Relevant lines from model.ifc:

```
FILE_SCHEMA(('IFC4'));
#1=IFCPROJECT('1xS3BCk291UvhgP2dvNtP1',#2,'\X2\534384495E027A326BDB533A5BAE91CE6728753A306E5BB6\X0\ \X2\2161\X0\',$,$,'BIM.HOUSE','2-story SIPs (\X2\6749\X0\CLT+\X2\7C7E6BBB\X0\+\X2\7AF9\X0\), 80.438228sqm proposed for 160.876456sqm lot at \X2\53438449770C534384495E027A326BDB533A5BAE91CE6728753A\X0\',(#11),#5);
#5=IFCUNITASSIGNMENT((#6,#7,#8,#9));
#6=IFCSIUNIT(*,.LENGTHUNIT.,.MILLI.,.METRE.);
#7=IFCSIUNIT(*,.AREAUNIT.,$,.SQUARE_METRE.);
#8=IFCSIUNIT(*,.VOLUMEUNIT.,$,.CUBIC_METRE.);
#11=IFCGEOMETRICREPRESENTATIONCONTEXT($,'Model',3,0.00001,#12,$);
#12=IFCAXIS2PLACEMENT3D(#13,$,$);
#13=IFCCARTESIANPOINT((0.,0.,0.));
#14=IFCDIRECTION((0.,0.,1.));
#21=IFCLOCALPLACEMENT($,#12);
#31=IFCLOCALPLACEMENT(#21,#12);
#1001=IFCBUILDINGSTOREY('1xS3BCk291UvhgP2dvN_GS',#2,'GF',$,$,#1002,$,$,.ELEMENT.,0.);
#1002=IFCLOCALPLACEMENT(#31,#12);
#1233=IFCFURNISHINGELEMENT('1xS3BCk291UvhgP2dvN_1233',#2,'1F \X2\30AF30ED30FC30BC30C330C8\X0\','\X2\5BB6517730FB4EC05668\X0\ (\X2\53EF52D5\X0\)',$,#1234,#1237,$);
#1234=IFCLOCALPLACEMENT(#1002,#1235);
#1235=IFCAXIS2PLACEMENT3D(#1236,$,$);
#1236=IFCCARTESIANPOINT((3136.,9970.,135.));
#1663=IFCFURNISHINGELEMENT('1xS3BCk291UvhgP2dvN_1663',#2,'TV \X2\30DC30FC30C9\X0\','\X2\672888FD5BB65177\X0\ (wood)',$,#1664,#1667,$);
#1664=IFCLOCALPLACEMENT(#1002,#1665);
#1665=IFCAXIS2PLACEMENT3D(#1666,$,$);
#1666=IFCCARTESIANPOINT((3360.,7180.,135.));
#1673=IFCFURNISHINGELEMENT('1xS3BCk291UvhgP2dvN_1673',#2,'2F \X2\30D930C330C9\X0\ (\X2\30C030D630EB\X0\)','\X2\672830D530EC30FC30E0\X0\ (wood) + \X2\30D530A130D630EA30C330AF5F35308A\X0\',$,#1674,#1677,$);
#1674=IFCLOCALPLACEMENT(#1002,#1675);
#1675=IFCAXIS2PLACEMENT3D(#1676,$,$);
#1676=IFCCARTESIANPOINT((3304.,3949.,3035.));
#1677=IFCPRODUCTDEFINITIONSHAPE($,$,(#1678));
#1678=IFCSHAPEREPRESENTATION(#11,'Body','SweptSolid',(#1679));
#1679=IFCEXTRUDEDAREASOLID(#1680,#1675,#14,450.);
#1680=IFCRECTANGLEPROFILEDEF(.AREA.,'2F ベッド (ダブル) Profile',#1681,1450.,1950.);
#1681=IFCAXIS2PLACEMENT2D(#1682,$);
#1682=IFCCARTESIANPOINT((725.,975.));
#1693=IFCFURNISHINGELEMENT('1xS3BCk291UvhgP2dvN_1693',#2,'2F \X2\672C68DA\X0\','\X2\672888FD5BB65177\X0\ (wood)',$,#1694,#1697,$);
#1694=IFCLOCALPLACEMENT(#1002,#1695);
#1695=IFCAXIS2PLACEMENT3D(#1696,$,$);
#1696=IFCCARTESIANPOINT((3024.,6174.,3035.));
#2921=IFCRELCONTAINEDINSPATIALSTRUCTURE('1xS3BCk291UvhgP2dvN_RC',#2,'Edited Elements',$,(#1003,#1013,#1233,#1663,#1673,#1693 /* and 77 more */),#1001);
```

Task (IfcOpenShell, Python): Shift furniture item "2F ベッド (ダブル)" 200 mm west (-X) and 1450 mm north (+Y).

```python
import ifcopenshell
import ifcopenshell.api.geometry
import ifcopenshell.util.placement
import ifcopenshell.util.unit

model = ifcopenshell.open("model.ifc")
unit_scale = ifcopenshell.util.unit.calculate_unit_scale(model)

item = model.by_guid("1xS3BCk291UvhgP2dvN_1673")
matrix = ifcopenshell.util.placement.get_local_placement(item.ObjectPlacement)
matrix[0, 3] -= 0.2 / unit_scale
matrix[1, 3] += 1.45 / unit_scale
ifcopenshell.api.geometry.edit_object_placement(model, product=item, matrix=matrix, is_si=False)

print(ifcopenshell.util.placement.get_local_placement(item.ObjectPlacement).round(3) + 0.0)

model.write("model_edited.ifc")
```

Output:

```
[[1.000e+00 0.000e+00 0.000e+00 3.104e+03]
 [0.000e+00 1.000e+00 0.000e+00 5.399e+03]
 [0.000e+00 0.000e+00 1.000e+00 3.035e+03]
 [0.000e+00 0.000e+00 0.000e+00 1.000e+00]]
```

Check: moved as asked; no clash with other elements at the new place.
